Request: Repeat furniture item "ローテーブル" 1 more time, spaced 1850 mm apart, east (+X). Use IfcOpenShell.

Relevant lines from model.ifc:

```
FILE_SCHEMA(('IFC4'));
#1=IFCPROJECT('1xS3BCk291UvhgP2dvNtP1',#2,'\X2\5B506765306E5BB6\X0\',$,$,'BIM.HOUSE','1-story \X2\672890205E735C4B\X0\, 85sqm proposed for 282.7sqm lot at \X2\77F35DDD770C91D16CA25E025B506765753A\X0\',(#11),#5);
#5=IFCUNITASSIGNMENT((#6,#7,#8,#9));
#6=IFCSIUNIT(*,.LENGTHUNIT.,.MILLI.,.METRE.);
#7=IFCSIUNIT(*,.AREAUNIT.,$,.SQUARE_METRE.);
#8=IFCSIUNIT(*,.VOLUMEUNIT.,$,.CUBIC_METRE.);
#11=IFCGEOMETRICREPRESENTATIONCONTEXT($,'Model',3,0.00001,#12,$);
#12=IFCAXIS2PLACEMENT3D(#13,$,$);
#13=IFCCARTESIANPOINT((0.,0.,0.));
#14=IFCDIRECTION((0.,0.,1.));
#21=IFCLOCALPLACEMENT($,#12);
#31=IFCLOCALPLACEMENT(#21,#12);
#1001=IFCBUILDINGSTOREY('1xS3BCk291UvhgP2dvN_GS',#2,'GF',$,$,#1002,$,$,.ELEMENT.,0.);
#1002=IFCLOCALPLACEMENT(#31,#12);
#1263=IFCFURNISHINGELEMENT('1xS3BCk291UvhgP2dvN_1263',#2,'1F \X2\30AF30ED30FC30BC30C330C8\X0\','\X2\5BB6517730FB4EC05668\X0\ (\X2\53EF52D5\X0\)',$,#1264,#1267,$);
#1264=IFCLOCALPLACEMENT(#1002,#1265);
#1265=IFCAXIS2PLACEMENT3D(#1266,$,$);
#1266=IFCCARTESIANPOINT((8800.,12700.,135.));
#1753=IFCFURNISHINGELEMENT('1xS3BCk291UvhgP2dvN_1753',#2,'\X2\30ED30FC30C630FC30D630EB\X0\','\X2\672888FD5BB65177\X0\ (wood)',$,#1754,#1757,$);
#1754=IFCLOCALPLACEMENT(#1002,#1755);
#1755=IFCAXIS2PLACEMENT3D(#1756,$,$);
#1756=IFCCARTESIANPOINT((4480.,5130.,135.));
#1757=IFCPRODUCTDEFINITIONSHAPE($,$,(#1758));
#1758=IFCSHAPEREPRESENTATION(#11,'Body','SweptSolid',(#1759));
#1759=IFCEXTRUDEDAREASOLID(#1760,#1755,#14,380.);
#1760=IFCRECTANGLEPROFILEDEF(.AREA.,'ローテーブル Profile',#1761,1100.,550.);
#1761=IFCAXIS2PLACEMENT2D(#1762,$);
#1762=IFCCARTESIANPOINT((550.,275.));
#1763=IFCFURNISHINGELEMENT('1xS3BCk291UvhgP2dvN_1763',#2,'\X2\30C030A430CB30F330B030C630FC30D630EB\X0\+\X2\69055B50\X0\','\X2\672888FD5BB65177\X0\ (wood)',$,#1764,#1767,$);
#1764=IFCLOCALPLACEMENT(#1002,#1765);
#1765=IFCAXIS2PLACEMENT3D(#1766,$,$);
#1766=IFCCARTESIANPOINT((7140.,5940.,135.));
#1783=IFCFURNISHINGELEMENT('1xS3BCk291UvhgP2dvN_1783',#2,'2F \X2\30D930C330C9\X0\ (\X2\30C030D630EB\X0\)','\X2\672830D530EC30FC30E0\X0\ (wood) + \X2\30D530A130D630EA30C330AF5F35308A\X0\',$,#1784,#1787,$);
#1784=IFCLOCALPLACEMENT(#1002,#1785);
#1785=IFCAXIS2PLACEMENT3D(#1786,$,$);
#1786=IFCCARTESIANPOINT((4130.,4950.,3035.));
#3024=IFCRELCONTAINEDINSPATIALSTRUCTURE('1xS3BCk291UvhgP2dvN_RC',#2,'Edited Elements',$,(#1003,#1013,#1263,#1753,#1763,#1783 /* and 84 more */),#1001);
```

```python
import numpy as np
import ifcopenshell
import ifcopenshell.api.geometry
import ifcopenshell.api.root
import ifcopenshell.util.element
import ifcopenshell.util.placement
import ifcopenshell.util.unit

model = ifcopenshell.open("model.ifc")
unit_scale = ifcopenshell.util.unit.calculate_unit_scale(model)


def reuse_history(source, copy):
    """copy_class also copies each property set's owner history, people and application; keep the originals."""
    for rel in copy.IsDefinedBy:
        if rel.is_a("IfcRelDefinesByProperties") and (history := rel.RelatingPropertyDefinition.OwnerHistory):
            rel.RelatingPropertyDefinition.OwnerHistory = source.OwnerHistory
            ifcopenshell.util.element.remove_deep2(model, history)


source = model.by_id(1753)
base = ifcopenshell.util.placement.get_local_placement(source.ObjectPlacement)
step = np.array([1.0, 0.0, 0.0]) * 1.85 / unit_scale

for i in range(1, 2):
    copy = ifcopenshell.api.root.copy_class(model, product=source)
    copy.Representation = ifcopenshell.util.element.copy_deep(
        model, source.Representation, exclude=["IfcGeometricRepresentationContext", "IfcRepresentationMap"]
    )
    reuse_history(source, copy)
    matrix = base.copy()
    matrix[:3, 3] += i * step
    print("added at", matrix[:3, 3].round(3) + 0.0)
    ifcopenshell.api.geometry.edit_object_placement(model, product=copy, matrix=matrix, is_si=False)

model.write("model_v2.ifc")
```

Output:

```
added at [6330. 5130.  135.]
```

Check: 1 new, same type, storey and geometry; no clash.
